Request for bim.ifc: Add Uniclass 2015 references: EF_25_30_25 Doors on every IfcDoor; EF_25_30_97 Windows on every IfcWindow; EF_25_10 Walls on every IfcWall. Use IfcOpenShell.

First a look at what the model holds.

```python
import ifcopenshell

model = ifcopenshell.open("bim.ifc")
print(model.schema)
print("classifications:", [c.Name for c in model.by_type("IfcClassification")])
for ifc_class in ("IfcDoor", "IfcRoof", "IfcStair", "IfcWall", "IfcWindow"):
    print(ifc_class, len(model.by_type(ifc_class)))
```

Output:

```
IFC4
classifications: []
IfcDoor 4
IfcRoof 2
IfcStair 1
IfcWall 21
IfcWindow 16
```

```python
import ifcopenshell
import ifcopenshell.api.classification

model = ifcopenshell.open("bim.ifc")

system = ifcopenshell.api.classification.add_classification(model, classification="Uniclass 2015")

codes = {
    "IfcDoor": ("EF_25_30_25", "Doors"),
    "IfcWindow": ("EF_25_30_97", "Windows"),
    "IfcWall": ("EF_25_10", "Walls"),
}
for ifc_class, (code, name) in codes.items():
    products = model.by_type(ifc_class)
    ifcopenshell.api.classification.add_reference(
        model, products=products, classification=system, identification=code, name=name
    )
    print(code, len(products))

model.write("bim_edited.ifc")
```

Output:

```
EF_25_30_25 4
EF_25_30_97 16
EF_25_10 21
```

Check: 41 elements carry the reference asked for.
